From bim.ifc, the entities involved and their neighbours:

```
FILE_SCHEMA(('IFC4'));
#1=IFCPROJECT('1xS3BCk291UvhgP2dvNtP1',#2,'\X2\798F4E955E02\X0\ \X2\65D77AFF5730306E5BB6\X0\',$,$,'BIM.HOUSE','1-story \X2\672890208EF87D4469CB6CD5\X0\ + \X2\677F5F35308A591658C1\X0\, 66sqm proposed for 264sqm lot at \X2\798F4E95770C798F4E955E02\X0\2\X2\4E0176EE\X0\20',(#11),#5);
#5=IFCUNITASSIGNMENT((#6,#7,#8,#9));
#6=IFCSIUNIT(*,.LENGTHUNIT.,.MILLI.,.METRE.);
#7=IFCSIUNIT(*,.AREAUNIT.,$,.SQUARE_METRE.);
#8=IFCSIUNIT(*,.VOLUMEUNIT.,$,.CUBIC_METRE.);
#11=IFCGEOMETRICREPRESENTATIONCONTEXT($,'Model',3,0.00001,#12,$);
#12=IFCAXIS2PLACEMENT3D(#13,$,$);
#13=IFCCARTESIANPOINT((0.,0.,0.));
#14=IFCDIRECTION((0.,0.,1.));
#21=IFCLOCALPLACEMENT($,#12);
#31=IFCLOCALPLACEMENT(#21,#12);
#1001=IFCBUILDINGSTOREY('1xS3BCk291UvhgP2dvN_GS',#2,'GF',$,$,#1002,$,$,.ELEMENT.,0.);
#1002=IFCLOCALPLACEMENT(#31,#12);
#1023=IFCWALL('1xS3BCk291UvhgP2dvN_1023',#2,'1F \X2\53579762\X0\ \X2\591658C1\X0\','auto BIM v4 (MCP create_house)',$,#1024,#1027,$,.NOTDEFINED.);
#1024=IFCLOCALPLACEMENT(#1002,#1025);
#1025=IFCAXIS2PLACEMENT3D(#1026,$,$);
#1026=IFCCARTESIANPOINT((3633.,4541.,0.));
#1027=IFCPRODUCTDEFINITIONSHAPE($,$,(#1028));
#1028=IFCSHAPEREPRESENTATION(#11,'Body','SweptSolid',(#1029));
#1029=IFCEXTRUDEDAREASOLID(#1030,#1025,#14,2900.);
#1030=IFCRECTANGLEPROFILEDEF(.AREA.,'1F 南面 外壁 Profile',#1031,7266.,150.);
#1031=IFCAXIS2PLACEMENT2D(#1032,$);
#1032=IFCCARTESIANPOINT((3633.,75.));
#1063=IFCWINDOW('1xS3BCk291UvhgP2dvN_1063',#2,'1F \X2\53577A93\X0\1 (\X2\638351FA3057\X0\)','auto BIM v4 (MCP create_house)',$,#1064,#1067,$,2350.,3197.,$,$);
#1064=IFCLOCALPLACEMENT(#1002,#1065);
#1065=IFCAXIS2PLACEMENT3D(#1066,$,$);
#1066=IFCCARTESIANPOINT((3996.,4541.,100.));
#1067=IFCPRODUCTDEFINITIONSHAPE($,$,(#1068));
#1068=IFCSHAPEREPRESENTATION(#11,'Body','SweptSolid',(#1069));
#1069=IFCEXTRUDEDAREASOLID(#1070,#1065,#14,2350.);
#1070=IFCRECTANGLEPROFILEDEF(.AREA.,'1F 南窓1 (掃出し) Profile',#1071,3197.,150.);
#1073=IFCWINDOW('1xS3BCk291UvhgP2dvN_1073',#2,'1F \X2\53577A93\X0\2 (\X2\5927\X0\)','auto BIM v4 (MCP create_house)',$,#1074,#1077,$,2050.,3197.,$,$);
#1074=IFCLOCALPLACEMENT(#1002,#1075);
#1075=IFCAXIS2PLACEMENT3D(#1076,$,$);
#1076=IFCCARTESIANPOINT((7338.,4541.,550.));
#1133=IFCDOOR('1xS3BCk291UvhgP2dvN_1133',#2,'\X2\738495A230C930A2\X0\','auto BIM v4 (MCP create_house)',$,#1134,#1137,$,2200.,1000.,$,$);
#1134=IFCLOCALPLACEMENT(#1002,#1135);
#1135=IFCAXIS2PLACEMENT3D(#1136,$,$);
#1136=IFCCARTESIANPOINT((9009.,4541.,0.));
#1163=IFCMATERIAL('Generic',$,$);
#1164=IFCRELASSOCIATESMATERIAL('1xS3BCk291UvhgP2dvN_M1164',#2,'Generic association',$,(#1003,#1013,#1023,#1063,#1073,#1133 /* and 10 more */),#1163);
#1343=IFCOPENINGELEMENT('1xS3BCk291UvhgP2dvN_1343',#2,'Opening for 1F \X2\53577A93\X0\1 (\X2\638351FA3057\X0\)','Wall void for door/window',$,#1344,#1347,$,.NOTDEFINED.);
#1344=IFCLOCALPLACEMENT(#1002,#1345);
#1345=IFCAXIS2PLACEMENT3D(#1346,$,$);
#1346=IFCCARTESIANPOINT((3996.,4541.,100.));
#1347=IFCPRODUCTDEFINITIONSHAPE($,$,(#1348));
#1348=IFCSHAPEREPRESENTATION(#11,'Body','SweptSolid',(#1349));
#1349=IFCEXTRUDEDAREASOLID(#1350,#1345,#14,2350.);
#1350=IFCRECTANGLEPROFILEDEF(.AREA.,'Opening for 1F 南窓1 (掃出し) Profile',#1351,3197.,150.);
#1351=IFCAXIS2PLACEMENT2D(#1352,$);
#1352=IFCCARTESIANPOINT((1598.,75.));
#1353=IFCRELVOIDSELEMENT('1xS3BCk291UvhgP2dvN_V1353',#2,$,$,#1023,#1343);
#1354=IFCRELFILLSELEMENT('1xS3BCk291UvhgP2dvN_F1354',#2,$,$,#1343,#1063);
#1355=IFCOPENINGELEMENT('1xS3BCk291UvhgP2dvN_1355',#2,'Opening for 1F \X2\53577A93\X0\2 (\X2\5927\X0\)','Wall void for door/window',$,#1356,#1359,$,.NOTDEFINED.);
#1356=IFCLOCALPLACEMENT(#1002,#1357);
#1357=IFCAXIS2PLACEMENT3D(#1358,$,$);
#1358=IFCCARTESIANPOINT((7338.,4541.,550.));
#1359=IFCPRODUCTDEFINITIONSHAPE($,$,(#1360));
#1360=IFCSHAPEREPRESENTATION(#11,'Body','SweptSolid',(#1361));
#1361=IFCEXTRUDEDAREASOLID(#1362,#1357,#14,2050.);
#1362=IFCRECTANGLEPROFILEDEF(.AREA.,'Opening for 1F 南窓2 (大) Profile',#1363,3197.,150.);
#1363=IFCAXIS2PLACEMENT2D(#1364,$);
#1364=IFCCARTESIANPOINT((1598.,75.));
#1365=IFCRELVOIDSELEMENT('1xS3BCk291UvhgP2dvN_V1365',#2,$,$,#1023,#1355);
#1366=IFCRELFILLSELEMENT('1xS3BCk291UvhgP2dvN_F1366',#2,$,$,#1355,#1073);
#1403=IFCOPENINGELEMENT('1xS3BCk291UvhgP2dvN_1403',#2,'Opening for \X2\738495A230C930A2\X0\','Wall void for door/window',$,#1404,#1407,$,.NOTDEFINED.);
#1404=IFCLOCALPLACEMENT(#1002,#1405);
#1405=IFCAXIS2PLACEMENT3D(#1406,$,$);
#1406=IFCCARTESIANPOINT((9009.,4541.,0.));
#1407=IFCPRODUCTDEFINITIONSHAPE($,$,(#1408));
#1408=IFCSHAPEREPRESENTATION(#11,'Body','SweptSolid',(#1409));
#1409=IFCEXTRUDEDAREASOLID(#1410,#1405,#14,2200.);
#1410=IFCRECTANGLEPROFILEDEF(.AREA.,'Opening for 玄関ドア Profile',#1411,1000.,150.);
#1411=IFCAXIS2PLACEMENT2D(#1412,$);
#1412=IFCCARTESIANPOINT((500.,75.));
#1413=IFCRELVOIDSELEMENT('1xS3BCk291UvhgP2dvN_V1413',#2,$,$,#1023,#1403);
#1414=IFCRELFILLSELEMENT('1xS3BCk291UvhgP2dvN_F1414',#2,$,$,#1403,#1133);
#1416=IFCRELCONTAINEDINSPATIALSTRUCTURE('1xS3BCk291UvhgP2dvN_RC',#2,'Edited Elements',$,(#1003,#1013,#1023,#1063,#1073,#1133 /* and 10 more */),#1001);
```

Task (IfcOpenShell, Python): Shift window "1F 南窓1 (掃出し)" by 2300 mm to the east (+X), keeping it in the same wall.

```python
import ifcopenshell
import ifcopenshell.api.geometry
import ifcopenshell.util.placement
import ifcopenshell.util.unit

model = ifcopenshell.open("bim.ifc")
unit_scale = ifcopenshell.util.unit.calculate_unit_scale(model)

window = model.by_guid("1xS3BCk291UvhgP2dvN_1063")
opening = window.FillsVoids[0].RelatingOpeningElement
wall = opening.VoidsElements[0].RelatingBuildingElement

wall_matrix = ifcopenshell.util.placement.get_local_placement(wall.ObjectPlacement)
shift = wall_matrix[:3, 0] * 2.3 / unit_scale
before = ifcopenshell.util.placement.get_local_placement(window.ObjectPlacement)[:3, 3].copy()

# The window is not placed relative to its opening, so move both.
for product in (opening, window):
    matrix = ifcopenshell.util.placement.get_local_placement(product.ObjectPlacement)
    matrix[:3, 3] += shift
    ifcopenshell.api.geometry.edit_object_placement(model, product=product, matrix=matrix, is_si=False)

after = ifcopenshell.util.placement.get_local_placement(window.ObjectPlacement)[:3, 3]
print("window moved by", (after - before).round(3) + 0.0)

model.write("bim_rev.ifc")
```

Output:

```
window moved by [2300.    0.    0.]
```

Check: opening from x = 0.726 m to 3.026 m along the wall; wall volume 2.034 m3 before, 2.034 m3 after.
